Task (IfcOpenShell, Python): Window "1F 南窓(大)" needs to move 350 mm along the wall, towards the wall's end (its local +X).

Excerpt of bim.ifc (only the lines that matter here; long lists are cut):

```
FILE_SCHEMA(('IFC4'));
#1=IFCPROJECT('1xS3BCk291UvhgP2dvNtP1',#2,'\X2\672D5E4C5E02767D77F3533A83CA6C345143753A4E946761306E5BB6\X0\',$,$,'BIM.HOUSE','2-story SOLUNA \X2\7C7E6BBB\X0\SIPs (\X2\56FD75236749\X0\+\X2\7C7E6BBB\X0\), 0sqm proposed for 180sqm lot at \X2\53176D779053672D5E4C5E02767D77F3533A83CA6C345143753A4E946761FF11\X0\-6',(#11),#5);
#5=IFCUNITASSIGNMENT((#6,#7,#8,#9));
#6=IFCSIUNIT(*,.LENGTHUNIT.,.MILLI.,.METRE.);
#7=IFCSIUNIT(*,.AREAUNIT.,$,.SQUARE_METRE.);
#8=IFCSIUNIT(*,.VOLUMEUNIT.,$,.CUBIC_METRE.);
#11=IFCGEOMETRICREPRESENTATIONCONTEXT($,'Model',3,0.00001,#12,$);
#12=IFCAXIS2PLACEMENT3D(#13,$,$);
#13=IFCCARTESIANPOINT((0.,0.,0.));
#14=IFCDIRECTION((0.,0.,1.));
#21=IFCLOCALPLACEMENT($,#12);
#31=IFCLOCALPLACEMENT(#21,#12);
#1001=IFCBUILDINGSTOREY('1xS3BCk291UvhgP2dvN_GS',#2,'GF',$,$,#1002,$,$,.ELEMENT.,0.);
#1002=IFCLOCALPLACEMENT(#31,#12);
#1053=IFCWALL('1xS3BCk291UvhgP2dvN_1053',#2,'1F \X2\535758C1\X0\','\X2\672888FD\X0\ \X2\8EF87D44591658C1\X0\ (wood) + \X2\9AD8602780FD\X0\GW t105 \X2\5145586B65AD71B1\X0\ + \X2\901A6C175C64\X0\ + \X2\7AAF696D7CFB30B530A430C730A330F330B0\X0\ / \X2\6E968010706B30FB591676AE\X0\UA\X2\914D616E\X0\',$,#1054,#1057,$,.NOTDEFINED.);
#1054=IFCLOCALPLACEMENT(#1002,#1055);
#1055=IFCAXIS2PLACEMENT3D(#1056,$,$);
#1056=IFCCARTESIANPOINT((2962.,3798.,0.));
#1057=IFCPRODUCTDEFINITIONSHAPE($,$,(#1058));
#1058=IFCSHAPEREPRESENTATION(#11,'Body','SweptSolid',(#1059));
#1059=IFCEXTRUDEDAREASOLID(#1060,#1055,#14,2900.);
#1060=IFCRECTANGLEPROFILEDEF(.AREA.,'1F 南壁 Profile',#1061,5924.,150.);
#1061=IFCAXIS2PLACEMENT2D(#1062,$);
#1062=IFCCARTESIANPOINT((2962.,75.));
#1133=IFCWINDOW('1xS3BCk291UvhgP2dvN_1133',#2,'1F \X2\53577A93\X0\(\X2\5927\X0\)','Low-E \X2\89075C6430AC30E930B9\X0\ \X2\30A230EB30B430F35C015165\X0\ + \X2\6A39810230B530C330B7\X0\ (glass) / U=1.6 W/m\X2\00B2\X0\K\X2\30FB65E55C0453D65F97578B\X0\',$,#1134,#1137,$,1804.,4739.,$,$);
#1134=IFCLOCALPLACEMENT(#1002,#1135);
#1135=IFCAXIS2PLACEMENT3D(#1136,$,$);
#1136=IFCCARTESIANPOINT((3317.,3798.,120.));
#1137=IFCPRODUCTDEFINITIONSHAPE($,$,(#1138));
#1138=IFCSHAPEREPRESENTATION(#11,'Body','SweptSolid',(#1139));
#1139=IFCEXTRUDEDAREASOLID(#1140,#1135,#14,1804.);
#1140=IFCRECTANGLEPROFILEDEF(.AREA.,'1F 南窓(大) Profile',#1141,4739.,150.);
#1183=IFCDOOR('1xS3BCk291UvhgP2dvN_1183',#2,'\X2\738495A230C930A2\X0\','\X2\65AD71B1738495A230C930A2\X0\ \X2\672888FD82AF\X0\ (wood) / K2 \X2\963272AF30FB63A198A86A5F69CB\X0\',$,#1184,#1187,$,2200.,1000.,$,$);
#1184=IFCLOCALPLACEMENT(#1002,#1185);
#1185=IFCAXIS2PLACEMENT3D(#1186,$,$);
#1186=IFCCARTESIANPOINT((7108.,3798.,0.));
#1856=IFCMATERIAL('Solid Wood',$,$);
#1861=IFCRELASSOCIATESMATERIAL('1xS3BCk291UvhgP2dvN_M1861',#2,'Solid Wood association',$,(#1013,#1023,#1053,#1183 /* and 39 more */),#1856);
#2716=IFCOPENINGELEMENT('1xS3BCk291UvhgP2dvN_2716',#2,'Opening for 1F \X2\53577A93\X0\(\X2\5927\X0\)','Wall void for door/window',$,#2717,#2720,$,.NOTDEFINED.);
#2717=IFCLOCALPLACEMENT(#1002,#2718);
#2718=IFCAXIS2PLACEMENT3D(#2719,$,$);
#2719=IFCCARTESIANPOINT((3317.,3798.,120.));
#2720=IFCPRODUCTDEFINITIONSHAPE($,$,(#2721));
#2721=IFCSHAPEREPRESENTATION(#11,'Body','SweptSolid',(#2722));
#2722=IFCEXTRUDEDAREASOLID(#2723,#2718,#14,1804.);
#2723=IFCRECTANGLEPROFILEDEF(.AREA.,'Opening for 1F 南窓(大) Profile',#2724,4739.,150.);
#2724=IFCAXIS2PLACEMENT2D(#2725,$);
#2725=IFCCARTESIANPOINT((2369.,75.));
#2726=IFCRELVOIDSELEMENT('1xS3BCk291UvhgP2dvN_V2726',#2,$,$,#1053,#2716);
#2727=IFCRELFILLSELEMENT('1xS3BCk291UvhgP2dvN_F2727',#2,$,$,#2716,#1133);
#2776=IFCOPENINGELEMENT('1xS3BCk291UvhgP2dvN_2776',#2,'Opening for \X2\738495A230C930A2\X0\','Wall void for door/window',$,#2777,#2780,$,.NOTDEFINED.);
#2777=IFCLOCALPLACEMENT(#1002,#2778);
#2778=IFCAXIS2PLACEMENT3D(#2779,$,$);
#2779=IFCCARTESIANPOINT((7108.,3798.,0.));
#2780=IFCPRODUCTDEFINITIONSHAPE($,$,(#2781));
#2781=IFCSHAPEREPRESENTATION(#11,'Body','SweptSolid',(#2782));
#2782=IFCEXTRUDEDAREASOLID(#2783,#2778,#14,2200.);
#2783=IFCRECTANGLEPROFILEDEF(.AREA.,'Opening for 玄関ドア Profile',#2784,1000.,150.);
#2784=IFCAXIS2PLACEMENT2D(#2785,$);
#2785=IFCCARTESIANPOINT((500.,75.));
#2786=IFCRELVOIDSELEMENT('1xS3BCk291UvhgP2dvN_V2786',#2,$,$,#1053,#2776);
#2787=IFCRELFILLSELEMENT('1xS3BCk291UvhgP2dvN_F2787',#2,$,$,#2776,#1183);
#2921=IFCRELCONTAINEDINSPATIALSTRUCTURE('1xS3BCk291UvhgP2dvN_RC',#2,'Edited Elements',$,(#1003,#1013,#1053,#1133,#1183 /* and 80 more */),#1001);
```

```python
import ifcopenshell
import ifcopenshell.api.geometry
import ifcopenshell.util.placement

model = ifcopenshell.open("bim.ifc")

window = model.by_guid("1xS3BCk291UvhgP2dvN_1133")
opening = window.FillsVoids[0].RelatingOpeningElement
wall = opening.VoidsElements[0].RelatingBuildingElement

wall_matrix = ifcopenshell.util.placement.get_local_placement(wall.ObjectPlacement)
shift = wall_matrix[:3, 0] * 350.0
before = ifcopenshell.util.placement.get_local_placement(window.ObjectPlacement)[:3, 3].copy()

# The window is not placed relative to its opening, so move both.
for product in (opening, window):
    matrix = ifcopenshell.util.placement.get_local_placement(product.ObjectPlacement)
    matrix[:3, 3] += shift
    ifcopenshell.api.geometry.edit_object_placement(model, product=product, matrix=matrix, is_si=False)

after = ifcopenshell.util.placement.get_local_placement(window.ObjectPlacement)[:3, 3]
print("window moved by", (after - before).round(3) + 0.0)

model.write("bim_rev.ifc")
```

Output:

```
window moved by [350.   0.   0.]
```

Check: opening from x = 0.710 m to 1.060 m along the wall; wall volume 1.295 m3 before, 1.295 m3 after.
